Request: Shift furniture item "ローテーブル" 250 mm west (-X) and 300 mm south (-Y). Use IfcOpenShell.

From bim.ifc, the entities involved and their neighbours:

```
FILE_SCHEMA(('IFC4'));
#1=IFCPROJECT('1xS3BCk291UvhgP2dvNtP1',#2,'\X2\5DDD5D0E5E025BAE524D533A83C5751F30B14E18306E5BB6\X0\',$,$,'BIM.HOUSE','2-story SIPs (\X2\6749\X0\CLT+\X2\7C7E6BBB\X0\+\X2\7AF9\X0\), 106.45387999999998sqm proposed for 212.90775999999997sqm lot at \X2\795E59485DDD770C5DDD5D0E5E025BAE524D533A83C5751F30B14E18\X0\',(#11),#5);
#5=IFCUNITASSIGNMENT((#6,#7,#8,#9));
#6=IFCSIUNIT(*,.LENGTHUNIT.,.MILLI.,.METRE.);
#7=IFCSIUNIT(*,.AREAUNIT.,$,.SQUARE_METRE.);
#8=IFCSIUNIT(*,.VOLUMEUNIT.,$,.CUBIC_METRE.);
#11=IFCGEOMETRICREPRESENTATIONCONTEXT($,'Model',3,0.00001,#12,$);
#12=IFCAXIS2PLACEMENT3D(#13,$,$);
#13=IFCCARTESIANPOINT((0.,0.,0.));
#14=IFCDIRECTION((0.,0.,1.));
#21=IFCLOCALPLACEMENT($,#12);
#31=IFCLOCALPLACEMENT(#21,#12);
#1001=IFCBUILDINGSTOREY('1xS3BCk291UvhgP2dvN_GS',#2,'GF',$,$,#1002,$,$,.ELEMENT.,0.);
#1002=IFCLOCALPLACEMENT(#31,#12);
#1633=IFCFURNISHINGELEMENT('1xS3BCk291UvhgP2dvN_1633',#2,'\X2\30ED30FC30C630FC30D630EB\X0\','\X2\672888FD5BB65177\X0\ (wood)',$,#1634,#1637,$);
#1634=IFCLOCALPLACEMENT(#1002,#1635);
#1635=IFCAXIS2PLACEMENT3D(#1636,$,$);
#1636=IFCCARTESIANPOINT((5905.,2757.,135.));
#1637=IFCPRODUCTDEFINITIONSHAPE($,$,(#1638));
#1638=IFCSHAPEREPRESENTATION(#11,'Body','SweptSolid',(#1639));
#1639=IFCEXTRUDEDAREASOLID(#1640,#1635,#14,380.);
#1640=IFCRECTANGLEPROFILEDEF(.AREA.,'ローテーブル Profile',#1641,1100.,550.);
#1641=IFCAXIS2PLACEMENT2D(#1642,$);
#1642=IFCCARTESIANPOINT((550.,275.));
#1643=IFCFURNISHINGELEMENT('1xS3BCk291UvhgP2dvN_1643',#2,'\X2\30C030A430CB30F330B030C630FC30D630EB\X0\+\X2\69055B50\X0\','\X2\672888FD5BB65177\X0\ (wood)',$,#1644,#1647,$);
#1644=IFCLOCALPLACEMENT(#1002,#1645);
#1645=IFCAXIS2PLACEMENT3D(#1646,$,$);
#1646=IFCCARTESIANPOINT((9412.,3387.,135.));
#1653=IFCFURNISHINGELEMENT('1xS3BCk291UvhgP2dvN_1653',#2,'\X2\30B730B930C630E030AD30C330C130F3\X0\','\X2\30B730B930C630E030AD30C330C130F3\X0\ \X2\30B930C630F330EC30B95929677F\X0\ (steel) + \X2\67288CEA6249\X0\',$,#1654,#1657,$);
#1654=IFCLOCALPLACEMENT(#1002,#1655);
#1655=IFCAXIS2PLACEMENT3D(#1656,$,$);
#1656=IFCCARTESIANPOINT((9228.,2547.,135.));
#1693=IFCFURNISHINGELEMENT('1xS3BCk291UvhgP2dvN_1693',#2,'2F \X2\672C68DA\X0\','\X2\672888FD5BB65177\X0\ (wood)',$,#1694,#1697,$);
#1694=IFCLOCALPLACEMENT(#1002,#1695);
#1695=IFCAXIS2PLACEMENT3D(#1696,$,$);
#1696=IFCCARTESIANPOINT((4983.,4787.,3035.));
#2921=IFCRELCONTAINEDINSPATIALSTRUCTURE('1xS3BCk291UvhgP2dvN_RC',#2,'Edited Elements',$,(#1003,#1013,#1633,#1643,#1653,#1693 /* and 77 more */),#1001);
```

```python
import ifcopenshell
import ifcopenshell.api.geometry
import ifcopenshell.util.placement
import ifcopenshell.util.unit

model = ifcopenshell.open("bim.ifc")
unit_scale = ifcopenshell.util.unit.calculate_unit_scale(model)

item = model.by_id(1633)
matrix = ifcopenshell.util.placement.get_local_placement(item.ObjectPlacement)
matrix[0, 3] -= 0.25 / unit_scale
matrix[1, 3] -= 0.3 / unit_scale
ifcopenshell.api.geometry.edit_object_placement(model, product=item, matrix=matrix, is_si=False)

print(ifcopenshell.util.placement.get_local_placement(item.ObjectPlacement).round(3) + 0.0)

model.write("bim_rev.ifc")
```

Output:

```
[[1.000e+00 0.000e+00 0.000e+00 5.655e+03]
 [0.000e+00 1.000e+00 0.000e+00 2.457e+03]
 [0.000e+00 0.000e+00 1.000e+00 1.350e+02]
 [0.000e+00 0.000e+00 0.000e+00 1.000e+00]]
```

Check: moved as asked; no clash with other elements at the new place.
